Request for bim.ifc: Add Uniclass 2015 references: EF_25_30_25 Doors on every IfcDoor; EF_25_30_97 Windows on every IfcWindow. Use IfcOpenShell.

First a look at what the model holds.

```python
import ifcopenshell

model = ifcopenshell.open("bim.ifc")
print(model.schema)
print("classifications:", [c.Name for c in model.by_type("IfcClassification")])
for ifc_class in ("IfcDoor", "IfcRoof", "IfcStair", "IfcWall", "IfcWindow"):
    print(ifc_class, len(model.by_type(ifc_class)))
```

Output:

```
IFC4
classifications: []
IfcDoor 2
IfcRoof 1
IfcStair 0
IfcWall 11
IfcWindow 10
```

```python
import ifcopenshell
import ifcopenshell.api.classification

model = ifcopenshell.open("bim.ifc")

system = ifcopenshell.api.classification.add_classification(model, classification="Uniclass 2015")

codes = {
    "IfcDoor": ("EF_25_30_25", "Doors"),
    "IfcWindow": ("EF_25_30_97", "Windows"),
}
for ifc_class, (code, name) in codes.items():
    products = model.by_type(ifc_class)
    ifcopenshell.api.classification.add_reference(
        model, products=products, classification=system, identification=code, name=name
    )
    print(code, len(products))

model.write("bim_v2.ifc")
```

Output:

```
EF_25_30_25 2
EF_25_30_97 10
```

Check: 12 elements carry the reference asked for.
